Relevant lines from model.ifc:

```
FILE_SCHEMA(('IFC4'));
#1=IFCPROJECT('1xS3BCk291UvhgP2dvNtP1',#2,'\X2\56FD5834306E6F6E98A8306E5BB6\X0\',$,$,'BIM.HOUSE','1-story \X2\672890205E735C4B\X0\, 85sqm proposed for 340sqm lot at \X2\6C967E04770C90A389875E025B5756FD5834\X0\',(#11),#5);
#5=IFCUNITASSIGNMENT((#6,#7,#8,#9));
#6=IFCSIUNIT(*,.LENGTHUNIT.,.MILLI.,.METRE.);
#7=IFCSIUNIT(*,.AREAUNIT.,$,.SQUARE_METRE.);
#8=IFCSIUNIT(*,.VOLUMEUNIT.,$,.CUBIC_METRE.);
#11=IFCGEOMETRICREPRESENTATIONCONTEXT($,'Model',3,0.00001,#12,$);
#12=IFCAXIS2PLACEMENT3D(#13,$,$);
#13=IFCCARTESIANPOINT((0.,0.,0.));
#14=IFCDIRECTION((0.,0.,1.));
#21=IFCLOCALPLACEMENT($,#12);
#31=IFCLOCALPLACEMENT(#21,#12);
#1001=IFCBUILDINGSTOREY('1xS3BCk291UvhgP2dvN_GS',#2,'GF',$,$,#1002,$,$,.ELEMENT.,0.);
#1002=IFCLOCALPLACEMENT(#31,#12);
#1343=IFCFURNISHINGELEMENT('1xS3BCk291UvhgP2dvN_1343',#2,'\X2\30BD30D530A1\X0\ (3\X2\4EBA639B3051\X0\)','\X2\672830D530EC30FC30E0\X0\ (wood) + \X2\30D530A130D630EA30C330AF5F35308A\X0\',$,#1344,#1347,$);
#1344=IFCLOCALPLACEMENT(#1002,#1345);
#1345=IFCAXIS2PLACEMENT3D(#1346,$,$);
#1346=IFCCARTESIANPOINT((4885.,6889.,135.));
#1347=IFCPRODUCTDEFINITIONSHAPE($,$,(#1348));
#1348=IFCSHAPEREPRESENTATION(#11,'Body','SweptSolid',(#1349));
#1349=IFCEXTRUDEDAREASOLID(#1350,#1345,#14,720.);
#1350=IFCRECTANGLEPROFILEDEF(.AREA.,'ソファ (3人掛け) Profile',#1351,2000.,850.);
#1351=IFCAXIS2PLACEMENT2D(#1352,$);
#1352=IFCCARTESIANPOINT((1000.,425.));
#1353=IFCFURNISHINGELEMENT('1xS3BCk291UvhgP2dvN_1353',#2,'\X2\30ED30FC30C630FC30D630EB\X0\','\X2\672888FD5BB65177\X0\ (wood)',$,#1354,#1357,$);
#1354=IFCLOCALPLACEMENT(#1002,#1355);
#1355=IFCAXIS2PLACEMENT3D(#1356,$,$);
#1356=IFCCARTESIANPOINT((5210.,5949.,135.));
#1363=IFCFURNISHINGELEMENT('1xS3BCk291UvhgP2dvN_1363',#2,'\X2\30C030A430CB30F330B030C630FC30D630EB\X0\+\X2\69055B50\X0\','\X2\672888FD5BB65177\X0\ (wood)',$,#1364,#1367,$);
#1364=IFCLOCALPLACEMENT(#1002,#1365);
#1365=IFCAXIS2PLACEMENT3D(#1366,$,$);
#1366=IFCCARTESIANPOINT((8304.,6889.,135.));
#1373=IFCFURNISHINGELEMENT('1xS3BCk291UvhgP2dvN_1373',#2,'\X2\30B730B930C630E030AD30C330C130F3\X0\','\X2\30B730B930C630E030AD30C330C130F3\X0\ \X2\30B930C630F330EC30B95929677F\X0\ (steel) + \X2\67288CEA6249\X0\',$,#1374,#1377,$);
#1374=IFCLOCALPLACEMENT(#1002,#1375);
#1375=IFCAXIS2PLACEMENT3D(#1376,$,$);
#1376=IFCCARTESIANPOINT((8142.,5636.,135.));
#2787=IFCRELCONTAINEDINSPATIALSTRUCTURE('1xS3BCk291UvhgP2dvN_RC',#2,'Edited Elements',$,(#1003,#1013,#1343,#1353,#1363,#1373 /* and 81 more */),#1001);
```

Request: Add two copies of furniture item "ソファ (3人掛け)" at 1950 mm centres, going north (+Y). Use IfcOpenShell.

```python
import numpy as np
import ifcopenshell
import ifcopenshell.api.geometry
import ifcopenshell.api.root
import ifcopenshell.util.element
import ifcopenshell.util.placement
import ifcopenshell.util.unit

model = ifcopenshell.open("model.ifc")
unit_scale = ifcopenshell.util.unit.calculate_unit_scale(model)


def reuse_history(source, copy):
    """copy_class also copies each property set's owner history, people and application; keep the originals."""
    for rel in copy.IsDefinedBy:
        if rel.is_a("IfcRelDefinesByProperties") and (history := rel.RelatingPropertyDefinition.OwnerHistory):
            rel.RelatingPropertyDefinition.OwnerHistory = source.OwnerHistory
            ifcopenshell.util.element.remove_deep2(model, history)


source = model.by_guid("1xS3BCk291UvhgP2dvN_1343")
base = ifcopenshell.util.placement.get_local_placement(source.ObjectPlacement)
step = np.array([0.0, 1.0, 0.0]) * 1.95 / unit_scale

for i in range(1, 3):
    copy = ifcopenshell.api.root.copy_class(model, product=source)
    copy.Representation = ifcopenshell.util.element.copy_deep(
        model, source.Representation, exclude=["IfcGeometricRepresentationContext", "IfcRepresentationMap"]
    )
    reuse_history(source, copy)
    matrix = base.copy()
    matrix[:3, 3] += i * step
    print("added at", matrix[:3, 3].round(3) + 0.0)
    ifcopenshell.api.geometry.edit_object_placement(model, product=copy, matrix=matrix, is_si=False)

model.write("model_v2.ifc")
```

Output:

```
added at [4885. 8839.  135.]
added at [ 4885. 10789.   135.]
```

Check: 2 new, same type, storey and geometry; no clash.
